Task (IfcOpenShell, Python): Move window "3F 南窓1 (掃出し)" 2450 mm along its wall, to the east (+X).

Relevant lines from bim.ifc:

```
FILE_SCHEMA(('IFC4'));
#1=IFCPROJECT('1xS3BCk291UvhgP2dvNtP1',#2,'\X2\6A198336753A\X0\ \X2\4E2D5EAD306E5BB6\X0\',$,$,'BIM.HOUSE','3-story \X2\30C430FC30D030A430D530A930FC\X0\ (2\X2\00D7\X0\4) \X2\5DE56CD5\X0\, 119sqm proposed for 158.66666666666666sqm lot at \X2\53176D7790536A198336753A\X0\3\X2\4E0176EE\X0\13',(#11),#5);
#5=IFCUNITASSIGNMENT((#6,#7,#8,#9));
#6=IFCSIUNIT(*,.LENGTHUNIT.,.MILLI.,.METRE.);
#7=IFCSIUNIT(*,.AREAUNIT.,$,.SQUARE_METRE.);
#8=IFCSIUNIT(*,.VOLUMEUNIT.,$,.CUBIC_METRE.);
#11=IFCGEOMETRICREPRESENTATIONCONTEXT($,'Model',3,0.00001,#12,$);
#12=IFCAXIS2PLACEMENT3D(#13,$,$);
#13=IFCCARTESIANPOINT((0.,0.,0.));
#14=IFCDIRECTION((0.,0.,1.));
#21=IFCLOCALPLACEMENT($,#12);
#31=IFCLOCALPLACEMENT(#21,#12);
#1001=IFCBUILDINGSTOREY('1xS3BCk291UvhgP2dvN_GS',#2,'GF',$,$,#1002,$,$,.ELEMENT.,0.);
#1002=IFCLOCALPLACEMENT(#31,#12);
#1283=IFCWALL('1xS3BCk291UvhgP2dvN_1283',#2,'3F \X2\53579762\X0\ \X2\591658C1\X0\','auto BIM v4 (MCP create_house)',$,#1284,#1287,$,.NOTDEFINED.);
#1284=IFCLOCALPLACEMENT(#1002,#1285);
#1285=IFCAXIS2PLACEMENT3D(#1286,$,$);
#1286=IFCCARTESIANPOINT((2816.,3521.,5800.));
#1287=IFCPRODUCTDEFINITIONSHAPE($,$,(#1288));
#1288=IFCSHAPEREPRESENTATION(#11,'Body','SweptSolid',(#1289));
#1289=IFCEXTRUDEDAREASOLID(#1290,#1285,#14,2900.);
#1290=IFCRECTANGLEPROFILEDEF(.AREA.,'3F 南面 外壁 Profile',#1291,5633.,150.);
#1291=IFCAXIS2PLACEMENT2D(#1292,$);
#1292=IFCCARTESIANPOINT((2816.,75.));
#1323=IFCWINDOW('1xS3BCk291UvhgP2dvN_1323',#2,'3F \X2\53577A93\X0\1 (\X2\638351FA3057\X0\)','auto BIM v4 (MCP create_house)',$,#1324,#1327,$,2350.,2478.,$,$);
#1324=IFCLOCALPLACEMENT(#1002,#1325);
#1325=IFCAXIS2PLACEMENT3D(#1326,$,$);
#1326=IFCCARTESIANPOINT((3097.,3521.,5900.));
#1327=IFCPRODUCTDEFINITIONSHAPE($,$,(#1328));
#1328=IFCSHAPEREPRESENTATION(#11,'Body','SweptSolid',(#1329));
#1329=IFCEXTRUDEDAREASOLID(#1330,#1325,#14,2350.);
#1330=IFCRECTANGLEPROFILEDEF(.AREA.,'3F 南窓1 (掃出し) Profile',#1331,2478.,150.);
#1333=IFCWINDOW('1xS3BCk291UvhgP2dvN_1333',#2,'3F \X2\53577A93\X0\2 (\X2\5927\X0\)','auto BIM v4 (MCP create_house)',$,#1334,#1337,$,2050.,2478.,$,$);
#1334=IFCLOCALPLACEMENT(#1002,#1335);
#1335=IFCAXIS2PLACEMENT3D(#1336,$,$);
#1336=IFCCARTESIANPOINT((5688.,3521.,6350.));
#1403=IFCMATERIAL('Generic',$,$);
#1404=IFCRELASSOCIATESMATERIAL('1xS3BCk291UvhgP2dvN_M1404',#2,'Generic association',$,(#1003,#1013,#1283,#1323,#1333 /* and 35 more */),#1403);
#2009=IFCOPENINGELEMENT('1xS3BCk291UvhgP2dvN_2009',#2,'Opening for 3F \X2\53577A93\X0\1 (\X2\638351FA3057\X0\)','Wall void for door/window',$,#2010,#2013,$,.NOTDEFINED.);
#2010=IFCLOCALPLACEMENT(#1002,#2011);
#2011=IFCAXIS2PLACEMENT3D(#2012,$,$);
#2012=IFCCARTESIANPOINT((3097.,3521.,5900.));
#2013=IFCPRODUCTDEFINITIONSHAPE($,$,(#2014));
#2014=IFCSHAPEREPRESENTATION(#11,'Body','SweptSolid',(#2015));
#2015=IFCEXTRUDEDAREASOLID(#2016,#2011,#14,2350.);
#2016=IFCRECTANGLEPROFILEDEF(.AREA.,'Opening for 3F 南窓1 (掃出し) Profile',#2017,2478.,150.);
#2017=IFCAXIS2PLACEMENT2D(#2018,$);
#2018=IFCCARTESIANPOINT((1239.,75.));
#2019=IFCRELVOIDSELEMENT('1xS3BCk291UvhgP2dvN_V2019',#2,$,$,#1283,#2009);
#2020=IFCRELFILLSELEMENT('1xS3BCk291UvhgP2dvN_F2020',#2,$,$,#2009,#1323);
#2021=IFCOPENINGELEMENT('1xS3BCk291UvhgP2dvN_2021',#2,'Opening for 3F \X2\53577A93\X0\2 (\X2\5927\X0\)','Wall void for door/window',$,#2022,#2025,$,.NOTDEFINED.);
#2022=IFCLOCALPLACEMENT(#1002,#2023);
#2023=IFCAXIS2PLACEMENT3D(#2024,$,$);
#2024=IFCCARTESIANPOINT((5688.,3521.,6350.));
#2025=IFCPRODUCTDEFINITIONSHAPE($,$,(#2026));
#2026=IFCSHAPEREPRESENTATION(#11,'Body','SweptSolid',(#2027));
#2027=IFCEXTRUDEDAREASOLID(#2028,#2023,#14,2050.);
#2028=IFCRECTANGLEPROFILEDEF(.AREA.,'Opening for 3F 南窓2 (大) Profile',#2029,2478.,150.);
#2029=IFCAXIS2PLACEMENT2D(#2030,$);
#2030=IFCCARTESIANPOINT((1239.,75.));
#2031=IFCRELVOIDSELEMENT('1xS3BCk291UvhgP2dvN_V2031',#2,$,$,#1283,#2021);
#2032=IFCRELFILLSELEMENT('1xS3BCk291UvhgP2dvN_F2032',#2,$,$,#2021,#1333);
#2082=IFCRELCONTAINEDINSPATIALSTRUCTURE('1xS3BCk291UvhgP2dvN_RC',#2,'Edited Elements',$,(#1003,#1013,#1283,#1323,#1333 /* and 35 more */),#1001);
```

```python
import ifcopenshell
import ifcopenshell.api.geometry
import ifcopenshell.util.placement

model = ifcopenshell.open("bim.ifc")

window = model.by_id(1323)
opening = window.FillsVoids[0].RelatingOpeningElement
wall = opening.VoidsElements[0].RelatingBuildingElement

wall_matrix = ifcopenshell.util.placement.get_local_placement(wall.ObjectPlacement)
shift = wall_matrix[:3, 0] * 2450.0
before = ifcopenshell.util.placement.get_local_placement(window.ObjectPlacement)[:3, 3].copy()

# The window is not placed relative to its opening, so move both.
for product in (opening, window):
    matrix = ifcopenshell.util.placement.get_local_placement(product.ObjectPlacement)
    matrix[:3, 3] += shift
    ifcopenshell.api.geometry.edit_object_placement(model, product=product, matrix=matrix, is_si=False)

after = ifcopenshell.util.placement.get_local_placement(window.ObjectPlacement)[:3, 3]
print("window moved by", (after - before).round(3) + 0.0)

model.write("bim_edited.ifc")
```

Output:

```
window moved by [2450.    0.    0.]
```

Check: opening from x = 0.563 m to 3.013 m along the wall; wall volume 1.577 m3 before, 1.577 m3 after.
